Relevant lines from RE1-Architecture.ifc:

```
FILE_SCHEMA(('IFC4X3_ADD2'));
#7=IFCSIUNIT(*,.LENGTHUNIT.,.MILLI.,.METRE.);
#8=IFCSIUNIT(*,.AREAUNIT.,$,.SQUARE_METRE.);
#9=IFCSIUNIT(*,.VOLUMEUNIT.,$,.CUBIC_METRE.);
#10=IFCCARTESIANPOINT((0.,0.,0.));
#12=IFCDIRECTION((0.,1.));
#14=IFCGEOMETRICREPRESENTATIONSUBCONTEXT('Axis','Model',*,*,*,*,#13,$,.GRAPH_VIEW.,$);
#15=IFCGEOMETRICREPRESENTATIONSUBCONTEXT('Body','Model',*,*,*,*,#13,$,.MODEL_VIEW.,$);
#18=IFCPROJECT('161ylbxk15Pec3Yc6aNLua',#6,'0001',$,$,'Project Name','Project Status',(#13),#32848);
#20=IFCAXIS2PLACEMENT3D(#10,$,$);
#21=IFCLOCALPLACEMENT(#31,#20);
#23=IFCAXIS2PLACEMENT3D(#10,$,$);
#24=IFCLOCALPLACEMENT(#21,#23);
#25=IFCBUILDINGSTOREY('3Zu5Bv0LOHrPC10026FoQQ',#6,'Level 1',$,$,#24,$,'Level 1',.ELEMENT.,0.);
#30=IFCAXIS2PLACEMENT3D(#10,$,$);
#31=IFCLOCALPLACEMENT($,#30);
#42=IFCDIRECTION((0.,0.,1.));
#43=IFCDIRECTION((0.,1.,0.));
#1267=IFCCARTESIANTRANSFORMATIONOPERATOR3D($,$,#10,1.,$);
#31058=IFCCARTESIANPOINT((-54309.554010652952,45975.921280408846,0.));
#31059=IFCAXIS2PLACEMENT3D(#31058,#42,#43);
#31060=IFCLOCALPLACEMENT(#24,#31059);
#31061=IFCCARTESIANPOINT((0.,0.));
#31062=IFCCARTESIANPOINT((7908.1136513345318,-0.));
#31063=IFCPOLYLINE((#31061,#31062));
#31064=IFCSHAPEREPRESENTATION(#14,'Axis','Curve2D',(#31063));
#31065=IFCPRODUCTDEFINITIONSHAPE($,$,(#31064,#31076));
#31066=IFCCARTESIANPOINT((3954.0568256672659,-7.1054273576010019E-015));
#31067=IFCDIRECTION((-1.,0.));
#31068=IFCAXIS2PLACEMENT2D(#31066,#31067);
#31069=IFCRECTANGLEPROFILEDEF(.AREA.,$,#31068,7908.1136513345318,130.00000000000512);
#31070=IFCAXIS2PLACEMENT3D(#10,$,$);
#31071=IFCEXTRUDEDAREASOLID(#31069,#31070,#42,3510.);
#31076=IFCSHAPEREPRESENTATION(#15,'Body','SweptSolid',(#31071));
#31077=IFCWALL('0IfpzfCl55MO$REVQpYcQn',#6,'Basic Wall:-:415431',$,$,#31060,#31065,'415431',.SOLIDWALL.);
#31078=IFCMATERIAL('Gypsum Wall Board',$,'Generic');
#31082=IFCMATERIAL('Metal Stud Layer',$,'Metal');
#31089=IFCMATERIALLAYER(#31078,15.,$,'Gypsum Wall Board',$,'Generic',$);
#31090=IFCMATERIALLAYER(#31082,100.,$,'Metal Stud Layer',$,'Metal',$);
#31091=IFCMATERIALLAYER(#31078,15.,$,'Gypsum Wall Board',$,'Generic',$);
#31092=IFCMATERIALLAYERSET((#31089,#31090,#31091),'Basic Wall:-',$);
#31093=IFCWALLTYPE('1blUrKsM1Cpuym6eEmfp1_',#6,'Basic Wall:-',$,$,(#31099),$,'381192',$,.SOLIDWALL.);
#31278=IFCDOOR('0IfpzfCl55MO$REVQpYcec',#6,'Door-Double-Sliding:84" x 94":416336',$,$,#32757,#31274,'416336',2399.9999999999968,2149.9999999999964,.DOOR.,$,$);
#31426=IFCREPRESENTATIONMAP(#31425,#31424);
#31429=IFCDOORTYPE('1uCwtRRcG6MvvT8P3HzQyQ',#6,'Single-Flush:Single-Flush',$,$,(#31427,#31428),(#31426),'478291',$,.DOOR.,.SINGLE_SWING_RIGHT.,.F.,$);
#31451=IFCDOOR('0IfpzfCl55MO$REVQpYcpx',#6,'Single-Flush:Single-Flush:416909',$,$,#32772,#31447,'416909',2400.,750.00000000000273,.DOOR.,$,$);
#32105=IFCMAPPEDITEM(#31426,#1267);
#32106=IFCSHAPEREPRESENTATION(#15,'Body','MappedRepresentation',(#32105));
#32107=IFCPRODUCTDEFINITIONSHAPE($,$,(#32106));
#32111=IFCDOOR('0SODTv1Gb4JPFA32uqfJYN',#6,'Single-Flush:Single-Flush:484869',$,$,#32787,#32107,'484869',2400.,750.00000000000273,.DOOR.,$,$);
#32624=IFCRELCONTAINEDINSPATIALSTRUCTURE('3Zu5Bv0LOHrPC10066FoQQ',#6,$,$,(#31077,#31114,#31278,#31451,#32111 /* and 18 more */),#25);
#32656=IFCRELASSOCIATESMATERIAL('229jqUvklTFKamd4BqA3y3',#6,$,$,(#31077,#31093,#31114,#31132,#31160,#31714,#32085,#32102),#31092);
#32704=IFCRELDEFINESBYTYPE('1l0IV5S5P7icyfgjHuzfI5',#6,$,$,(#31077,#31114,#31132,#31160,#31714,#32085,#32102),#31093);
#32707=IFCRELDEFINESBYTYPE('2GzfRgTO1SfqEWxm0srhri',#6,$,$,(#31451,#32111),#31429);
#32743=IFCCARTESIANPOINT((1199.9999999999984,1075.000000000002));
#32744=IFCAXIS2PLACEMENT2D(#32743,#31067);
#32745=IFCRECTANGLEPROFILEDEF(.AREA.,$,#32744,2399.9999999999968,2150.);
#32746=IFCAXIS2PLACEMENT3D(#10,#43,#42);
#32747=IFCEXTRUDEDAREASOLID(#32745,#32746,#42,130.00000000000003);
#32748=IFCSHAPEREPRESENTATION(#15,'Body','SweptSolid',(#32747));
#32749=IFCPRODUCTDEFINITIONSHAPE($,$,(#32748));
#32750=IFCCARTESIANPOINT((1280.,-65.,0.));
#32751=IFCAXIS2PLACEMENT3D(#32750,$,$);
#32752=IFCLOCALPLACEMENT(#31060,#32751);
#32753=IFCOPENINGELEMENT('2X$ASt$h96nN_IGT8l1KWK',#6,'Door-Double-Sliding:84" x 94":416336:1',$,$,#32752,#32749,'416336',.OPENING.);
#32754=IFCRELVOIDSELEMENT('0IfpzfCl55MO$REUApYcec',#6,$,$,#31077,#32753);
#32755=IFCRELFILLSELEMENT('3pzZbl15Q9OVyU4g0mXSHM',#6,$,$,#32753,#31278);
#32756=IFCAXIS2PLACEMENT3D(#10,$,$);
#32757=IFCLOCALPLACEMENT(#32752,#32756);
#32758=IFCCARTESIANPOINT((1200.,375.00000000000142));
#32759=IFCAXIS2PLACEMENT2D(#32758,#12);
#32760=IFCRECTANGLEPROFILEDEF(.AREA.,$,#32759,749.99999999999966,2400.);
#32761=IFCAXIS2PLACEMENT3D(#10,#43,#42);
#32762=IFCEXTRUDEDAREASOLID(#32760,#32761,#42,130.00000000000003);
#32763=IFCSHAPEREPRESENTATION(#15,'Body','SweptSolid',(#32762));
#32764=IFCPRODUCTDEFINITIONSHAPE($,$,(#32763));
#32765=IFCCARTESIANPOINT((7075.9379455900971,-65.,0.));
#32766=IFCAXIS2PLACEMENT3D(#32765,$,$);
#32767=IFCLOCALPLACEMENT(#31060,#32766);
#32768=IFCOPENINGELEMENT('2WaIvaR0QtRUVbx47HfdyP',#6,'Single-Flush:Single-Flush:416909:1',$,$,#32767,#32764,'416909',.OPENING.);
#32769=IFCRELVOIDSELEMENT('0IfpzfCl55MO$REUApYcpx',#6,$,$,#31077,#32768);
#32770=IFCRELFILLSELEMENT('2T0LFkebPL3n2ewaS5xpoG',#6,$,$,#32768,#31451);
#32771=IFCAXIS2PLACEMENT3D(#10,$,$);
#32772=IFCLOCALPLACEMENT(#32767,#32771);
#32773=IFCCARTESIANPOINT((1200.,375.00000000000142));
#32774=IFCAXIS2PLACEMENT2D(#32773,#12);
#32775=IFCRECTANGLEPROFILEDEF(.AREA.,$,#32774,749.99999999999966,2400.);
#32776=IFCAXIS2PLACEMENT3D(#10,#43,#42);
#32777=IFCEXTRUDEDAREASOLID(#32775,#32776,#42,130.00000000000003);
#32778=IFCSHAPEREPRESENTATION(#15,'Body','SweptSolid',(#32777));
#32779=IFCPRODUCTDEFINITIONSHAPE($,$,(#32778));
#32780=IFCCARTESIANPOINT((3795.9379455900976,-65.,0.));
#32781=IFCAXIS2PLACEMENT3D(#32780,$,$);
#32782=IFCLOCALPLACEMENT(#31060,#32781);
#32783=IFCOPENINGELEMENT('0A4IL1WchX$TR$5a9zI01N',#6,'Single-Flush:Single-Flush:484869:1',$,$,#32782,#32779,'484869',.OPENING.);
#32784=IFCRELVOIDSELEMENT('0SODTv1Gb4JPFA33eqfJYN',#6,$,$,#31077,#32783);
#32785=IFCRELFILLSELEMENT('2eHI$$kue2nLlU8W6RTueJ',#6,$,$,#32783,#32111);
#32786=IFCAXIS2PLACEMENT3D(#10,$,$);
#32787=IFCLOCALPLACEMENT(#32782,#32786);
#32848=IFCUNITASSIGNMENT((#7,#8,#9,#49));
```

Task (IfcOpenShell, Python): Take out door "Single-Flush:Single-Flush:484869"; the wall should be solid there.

```python
import ifcopenshell
import ifcopenshell.api.feature
import ifcopenshell.api.root
import ifcopenshell.geom
import ifcopenshell.util.shape

model = ifcopenshell.open("RE1-Architecture.ifc")
settings = ifcopenshell.geom.settings()


def volume(element):
    """Net volume in cubic metres, openings subtracted."""
    shape = ifcopenshell.geom.create_shape(settings, element)
    return ifcopenshell.util.shape.get_volume(shape.geometry)


door = model.by_id(32111)
opening = door.FillsVoids[0].RelatingOpeningElement
wall = opening.VoidsElements[0].RelatingBuildingElement
before = volume(wall)

ifcopenshell.api.root.remove_product(model, product=door)
ifcopenshell.api.feature.remove_feature(model, feature=opening)

after = volume(wall)

print(f"wall volume {before:.3f} -> {after:.3f} m3")

model.write("RE1-Architecture_updated.ifc")
```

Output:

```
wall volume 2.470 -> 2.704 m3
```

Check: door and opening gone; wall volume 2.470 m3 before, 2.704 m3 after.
